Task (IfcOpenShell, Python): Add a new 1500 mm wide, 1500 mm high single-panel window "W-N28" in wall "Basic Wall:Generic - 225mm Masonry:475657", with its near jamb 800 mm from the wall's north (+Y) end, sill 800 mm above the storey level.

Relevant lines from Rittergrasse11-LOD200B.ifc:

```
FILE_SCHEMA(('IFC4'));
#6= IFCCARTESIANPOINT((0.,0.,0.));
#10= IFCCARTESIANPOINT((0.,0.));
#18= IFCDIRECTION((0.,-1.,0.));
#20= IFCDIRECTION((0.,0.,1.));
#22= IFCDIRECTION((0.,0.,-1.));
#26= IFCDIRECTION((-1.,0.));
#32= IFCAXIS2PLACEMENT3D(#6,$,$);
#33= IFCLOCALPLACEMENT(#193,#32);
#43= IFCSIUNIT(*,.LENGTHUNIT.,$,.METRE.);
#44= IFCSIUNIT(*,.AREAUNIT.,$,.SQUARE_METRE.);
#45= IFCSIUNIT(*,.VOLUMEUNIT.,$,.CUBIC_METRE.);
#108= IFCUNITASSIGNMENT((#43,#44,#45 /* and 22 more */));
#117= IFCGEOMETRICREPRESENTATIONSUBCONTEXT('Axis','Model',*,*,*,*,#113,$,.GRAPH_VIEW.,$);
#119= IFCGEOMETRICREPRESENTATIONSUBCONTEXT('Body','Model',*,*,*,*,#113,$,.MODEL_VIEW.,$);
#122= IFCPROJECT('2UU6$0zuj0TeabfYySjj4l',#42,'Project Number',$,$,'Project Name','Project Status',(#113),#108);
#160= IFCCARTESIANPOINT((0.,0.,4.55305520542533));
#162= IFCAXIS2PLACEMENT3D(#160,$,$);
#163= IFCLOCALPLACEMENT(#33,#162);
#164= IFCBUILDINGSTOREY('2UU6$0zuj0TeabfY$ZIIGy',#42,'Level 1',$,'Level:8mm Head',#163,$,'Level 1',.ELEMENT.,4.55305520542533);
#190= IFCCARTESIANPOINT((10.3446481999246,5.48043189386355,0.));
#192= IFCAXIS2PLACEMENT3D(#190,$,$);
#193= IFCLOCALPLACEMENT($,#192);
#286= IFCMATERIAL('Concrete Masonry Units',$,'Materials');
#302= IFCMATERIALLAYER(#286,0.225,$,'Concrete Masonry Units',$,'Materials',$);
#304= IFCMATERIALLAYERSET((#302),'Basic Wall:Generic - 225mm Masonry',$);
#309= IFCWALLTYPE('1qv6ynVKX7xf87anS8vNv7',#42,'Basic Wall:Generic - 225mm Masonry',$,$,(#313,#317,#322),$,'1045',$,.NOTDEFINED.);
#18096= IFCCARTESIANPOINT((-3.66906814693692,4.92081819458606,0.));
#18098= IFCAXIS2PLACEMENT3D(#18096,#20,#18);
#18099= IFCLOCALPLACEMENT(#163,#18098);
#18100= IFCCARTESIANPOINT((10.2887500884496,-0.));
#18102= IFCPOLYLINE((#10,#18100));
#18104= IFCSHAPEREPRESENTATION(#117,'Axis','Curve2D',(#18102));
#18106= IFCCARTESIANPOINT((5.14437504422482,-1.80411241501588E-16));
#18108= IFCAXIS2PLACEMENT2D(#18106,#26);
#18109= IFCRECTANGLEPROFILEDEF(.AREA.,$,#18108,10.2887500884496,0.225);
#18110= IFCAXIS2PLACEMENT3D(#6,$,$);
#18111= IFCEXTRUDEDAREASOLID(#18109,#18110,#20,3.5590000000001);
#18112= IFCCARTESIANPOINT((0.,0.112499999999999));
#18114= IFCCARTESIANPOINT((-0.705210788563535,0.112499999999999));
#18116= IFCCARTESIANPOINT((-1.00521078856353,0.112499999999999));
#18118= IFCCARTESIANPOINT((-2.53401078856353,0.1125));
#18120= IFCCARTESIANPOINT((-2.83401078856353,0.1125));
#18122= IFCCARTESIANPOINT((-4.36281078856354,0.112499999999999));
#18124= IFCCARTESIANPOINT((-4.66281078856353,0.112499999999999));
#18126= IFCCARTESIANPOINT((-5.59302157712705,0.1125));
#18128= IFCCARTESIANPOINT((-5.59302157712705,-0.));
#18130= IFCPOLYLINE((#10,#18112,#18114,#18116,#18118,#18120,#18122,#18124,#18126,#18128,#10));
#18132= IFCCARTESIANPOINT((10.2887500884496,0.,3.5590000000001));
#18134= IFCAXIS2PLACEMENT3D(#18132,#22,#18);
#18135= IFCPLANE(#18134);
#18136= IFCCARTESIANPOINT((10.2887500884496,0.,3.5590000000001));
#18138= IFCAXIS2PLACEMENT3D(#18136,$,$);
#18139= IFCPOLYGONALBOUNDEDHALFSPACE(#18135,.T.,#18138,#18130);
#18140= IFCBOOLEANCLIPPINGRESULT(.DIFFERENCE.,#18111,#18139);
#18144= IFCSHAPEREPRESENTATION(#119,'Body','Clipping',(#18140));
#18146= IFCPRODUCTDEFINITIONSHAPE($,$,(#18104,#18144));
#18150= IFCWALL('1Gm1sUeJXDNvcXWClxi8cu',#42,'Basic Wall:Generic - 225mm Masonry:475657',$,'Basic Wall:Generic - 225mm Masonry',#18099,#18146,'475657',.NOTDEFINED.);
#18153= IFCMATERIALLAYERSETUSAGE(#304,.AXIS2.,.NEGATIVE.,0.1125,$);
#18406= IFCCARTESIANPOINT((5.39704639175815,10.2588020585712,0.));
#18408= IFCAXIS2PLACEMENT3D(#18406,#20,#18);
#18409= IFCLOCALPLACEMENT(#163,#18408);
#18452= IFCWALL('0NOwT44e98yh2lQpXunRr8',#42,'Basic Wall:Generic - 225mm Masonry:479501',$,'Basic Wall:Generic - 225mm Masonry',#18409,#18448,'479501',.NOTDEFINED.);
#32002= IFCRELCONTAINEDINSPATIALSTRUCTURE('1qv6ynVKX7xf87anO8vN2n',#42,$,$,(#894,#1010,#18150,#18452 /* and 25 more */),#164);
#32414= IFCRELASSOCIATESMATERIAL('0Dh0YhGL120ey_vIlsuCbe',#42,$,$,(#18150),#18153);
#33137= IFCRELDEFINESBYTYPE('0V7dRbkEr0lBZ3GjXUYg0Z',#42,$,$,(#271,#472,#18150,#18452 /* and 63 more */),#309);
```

```python
import numpy as np
import ifcopenshell
import ifcopenshell.api.feature
import ifcopenshell.api.geometry
import ifcopenshell.api.root
import ifcopenshell.api.spatial
import ifcopenshell.geom
import ifcopenshell.util.element
import ifcopenshell.util.placement
import ifcopenshell.util.representation
import ifcopenshell.util.shape
import ifcopenshell.util.unit

model = ifcopenshell.open("Rittergrasse11-LOD200B.ifc")
unit_scale = ifcopenshell.util.unit.calculate_unit_scale(model)
settings = ifcopenshell.geom.settings()


def volume(element):
    """Net volume in cubic metres, openings subtracted."""
    shape = ifcopenshell.geom.create_shape(settings, element)
    return ifcopenshell.util.shape.get_volume(shape.geometry)


wall = model.by_id(18150)
storey = ifcopenshell.util.element.get_container(wall, ifc_class="IfcBuildingStorey")
context = ifcopenshell.util.representation.get_context(model, "Model", "Body", "MODEL_VIEW")
before = volume(wall)

width, height, from_end, sill = 1.5, 1.5, 0.8, 0.8  # metres

# The wall runs along its own X axis, and the end named is its -X end.
wall_shape = ifcopenshell.geom.create_shape(settings, wall)
x, y, z = ifcopenshell.util.shape.get_vertices(wall_shape.geometry).T
start = x.min() + from_end
face, thickness = float(y.min()), float(y.max() - y.min())
wall_matrix = ifcopenshell.util.placement.get_local_placement(wall.ObjectPlacement)
level = ifcopenshell.util.placement.get_local_placement(storey.ObjectPlacement)[2, 3]


def in_wall(x, y):
    """Placement at x, y metres in the wall's axes, at sill height."""
    matrix = wall_matrix.copy()
    matrix[:, 3] = wall_matrix @ np.array([x / unit_scale, y / unit_scale, 0.0, 1.0])
    matrix[2, 3] = level + sill / unit_scale
    return matrix


# Opening: a box that overshoots both wall faces by 50 mm.
opening = ifcopenshell.api.root.create_entity(model, ifc_class="IfcOpeningElement", predefined_type="OPENING")
box = ifcopenshell.api.geometry.add_wall_representation(
    model, context=context, length=width, height=height, thickness=thickness + 0.1
)
ifcopenshell.api.geometry.assign_representation(model, product=opening, representation=box)
ifcopenshell.api.geometry.edit_object_placement(model, product=opening, matrix=in_wall(start, face - 0.05), is_si=False)
ifcopenshell.api.feature.add_feature(model, feature=opening, element=wall)

window = ifcopenshell.api.root.create_entity(model, ifc_class="IfcWindow", name="W-N28", predefined_type="WINDOW")
window.OverallWidth, window.OverallHeight = width / unit_scale, height / unit_scale
window.PartitioningType = "SINGLE_PANEL"
body = ifcopenshell.api.geometry.add_window_representation(
    model,
    context=context,
    overall_width=window.OverallWidth,
    overall_height=window.OverallHeight,
    partition_type="SINGLE_PANEL",
)
ifcopenshell.api.geometry.assign_representation(model, product=window, representation=body)
ifcopenshell.api.spatial.assign_container(model, products=[window], relating_structure=storey)
ifcopenshell.api.feature.add_filling(model, opening=opening, element=window)

# Centre the window in the wall's thickness.
ifcopenshell.api.geometry.edit_object_placement(model, product=window, matrix=in_wall(start, face), is_si=False)
window_shape = ifcopenshell.geom.create_shape(settings, window)
depth = ifcopenshell.util.shape.get_vertices(window_shape.geometry)[:, 1]
offset = face + thickness / 2 - (depth.min() + depth.max()) / 2
ifcopenshell.api.geometry.edit_object_placement(model, product=window, matrix=in_wall(start, offset), is_si=False)

after = volume(wall)

print(f"wall volume {before:.3f} -> {after:.3f} m3")

model.write("Rittergrasse11-LOD200B-out.ifc")
```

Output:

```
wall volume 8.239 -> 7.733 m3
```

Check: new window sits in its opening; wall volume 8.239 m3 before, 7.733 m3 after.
